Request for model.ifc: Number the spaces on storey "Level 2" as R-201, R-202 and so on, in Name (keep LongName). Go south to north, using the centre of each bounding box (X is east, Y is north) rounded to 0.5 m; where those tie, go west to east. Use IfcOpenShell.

First a look at what the model holds.

```python
import ifcopenshell
import ifcopenshell.util.element
import ifcopenshell.util.placement

model = ifcopenshell.open("model.ifc")
print(model.schema)
storey = next(s for s in model.by_type("IfcBuildingStorey") if s.Name == "Level 2")
spaces = [e for e in ifcopenshell.util.element.get_decomposition(storey) if e.is_a("IfcSpace")]
for e in sorted(spaces, key=lambda e: e.id()):
    origin = ifcopenshell.util.placement.get_local_placement(e.ObjectPlacement)[:3, 3]
    print(e.id(), e.Name, e.LongName, origin.round(2) + 0.0, sep=" | ")
```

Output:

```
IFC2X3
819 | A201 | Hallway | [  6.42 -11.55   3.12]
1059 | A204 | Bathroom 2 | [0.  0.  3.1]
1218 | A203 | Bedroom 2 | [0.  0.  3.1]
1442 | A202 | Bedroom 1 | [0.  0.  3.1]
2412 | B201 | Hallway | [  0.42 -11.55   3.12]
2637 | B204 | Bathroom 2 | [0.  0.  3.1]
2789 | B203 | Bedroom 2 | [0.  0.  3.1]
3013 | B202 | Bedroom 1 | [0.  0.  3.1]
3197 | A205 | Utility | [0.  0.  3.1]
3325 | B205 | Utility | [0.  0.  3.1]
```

```python
import ifcopenshell
import ifcopenshell.geom
import ifcopenshell.util.element
import ifcopenshell.util.shape

model = ifcopenshell.open("model.ifc")
settings = ifcopenshell.geom.settings()
settings.set("use-world-coords", True)


def centre(element):
    shape = ifcopenshell.geom.create_shape(settings, element)
    return ifcopenshell.util.shape.get_bbox_centroid(shape.geometry)


storey = next(s for s in model.by_type("IfcBuildingStorey") if s.Name == "Level 2")
spaces = [e for e in ifcopenshell.util.element.get_decomposition(storey) if e.is_a("IfcSpace")]

# Insertion points can sit at a corner or the storey origin, so sort by the geometry (in metres).
centres = {e: centre(e) for e in spaces}
spaces.sort(key=lambda e: (round(centres[e][1] / 0.5), centres[e][0]))

for i, e in enumerate(spaces, start=1):
    number = f"R-2{i:02d}"
    e.Name = number
    print(e.id(), number)

model.write("model_updated.ifc")
```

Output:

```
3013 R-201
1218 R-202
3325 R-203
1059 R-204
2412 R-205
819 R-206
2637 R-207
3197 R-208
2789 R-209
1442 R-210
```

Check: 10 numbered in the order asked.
